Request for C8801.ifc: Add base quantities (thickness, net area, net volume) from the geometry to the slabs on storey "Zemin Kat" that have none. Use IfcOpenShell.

First a look at what the model holds.

```python
import ifcopenshell
import ifcopenshell.util.element
import ifcopenshell.util.unit

model = ifcopenshell.open("C8801.ifc")
print(model.schema)
for unit_type in ("LENGTHUNIT", "AREAUNIT", "VOLUMEUNIT"):
    print(unit_type, ifcopenshell.util.unit.calculate_unit_scale(model, unit_type))
storey = next(s for s in model.by_type("IfcBuildingStorey") if s.Name == "Zemin Kat")
slabs = [e for e in ifcopenshell.util.element.get_decomposition(storey) if e.is_a("IfcSlab")]
for e in sorted(slabs, key=lambda e: e.id()):
    print(e.id(), e.is_a(), e.Name, list(ifcopenshell.util.element.get_psets(e, qtos_only=True)), sep=" | ")
```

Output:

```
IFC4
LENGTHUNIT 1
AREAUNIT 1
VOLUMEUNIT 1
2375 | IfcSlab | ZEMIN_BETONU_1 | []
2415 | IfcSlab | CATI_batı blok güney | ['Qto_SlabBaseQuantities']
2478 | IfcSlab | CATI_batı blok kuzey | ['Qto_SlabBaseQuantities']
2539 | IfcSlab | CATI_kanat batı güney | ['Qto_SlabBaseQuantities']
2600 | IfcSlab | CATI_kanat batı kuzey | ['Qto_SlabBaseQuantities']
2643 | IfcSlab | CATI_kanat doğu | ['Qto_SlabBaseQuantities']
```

```python
import ifcopenshell
import ifcopenshell.api.pset
import ifcopenshell.geom
import ifcopenshell.util.element
import ifcopenshell.util.shape
import ifcopenshell.util.unit

model = ifcopenshell.open("C8801.ifc")
unit_scale = ifcopenshell.util.unit.calculate_unit_scale(model)
area_scale = ifcopenshell.util.unit.calculate_unit_scale(model, "AREAUNIT")
volume_scale = ifcopenshell.util.unit.calculate_unit_scale(model, "VOLUMEUNIT")
settings = ifcopenshell.geom.settings()

storey = next(s for s in model.by_type("IfcBuildingStorey") if s.Name == "Zemin Kat")
slabs = [e for e in ifcopenshell.util.element.get_decomposition(storey) if e.is_a("IfcSlab")]

for e in sorted(slabs, key=lambda e: e.id()):
    if ifcopenshell.util.element.get_psets(e, qtos_only=True, should_inherit=False):
        continue
    # Geometry comes back in metres, in the element's own axes.
    shape = ifcopenshell.geom.create_shape(settings, e)
    values = {
        "Width": ifcopenshell.util.shape.get_z(shape.geometry) / unit_scale,
        "NetArea": ifcopenshell.util.shape.get_footprint_area(shape.geometry) / area_scale,
        "NetVolume": ifcopenshell.util.shape.get_volume(shape.geometry) / volume_scale,
    }
    qto = ifcopenshell.api.pset.add_qto(model, product=e, name="Qto_SlabBaseQuantities")
    ifcopenshell.api.pset.edit_qto(model, qto=qto, properties=values)
    print(e.id(), {k: round(v, 3) for k, v in values.items()})

model.write("C8801_rev.ifc")
```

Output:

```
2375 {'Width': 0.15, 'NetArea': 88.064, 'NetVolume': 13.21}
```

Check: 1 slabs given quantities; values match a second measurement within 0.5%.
